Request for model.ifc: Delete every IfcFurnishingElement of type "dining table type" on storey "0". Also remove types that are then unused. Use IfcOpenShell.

First a look at what the model holds.

```python
import ifcopenshell
import ifcopenshell.util.element

model = ifcopenshell.open("model.ifc")
print(model.schema)
storey = next(s for s in model.by_type("IfcBuildingStorey") if s.Name == "0")
furniture = [e for e in ifcopenshell.util.element.get_decomposition(storey) if e.is_a("IfcFurnishingElement")]
seen = {}
for e in furniture:
    element_type = ifcopenshell.util.element.get_type(e)
    name = element_type.Name if element_type not in (None, e) else None
    seen[name] = seen.get(name, 0) + 1
for name, count in sorted(seen.items(), key=str):
    print(count, "x", name)
```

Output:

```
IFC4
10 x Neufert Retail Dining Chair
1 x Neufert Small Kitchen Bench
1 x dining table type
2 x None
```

```python
import ifcopenshell
import ifcopenshell.api.root
import ifcopenshell.util.element

model = ifcopenshell.open("model.ifc")

storey = next(s for s in model.by_type("IfcBuildingStorey") if s.Name == "0")
furniture = [e for e in ifcopenshell.util.element.get_decomposition(storey) if e.is_a("IfcFurnishingElement")]
targets = [e for e in furniture if (t := ifcopenshell.util.element.get_type(e)) not in (None, e) and t.Name == "dining table type"]
types = {ifcopenshell.util.element.get_type(e) for e in targets} - {None, *targets}

for e in targets:
    ifcopenshell.api.root.remove_product(model, product=e)
print(len(targets), "removed")

unused = [t for t in types if not ifcopenshell.util.element.get_types(t)]
for t in unused:
    ifcopenshell.api.root.remove_product(model, product=t)
print(len(unused), "unused types removed")

model.write("model_rev.ifc")
```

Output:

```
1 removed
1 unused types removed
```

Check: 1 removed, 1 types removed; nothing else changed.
